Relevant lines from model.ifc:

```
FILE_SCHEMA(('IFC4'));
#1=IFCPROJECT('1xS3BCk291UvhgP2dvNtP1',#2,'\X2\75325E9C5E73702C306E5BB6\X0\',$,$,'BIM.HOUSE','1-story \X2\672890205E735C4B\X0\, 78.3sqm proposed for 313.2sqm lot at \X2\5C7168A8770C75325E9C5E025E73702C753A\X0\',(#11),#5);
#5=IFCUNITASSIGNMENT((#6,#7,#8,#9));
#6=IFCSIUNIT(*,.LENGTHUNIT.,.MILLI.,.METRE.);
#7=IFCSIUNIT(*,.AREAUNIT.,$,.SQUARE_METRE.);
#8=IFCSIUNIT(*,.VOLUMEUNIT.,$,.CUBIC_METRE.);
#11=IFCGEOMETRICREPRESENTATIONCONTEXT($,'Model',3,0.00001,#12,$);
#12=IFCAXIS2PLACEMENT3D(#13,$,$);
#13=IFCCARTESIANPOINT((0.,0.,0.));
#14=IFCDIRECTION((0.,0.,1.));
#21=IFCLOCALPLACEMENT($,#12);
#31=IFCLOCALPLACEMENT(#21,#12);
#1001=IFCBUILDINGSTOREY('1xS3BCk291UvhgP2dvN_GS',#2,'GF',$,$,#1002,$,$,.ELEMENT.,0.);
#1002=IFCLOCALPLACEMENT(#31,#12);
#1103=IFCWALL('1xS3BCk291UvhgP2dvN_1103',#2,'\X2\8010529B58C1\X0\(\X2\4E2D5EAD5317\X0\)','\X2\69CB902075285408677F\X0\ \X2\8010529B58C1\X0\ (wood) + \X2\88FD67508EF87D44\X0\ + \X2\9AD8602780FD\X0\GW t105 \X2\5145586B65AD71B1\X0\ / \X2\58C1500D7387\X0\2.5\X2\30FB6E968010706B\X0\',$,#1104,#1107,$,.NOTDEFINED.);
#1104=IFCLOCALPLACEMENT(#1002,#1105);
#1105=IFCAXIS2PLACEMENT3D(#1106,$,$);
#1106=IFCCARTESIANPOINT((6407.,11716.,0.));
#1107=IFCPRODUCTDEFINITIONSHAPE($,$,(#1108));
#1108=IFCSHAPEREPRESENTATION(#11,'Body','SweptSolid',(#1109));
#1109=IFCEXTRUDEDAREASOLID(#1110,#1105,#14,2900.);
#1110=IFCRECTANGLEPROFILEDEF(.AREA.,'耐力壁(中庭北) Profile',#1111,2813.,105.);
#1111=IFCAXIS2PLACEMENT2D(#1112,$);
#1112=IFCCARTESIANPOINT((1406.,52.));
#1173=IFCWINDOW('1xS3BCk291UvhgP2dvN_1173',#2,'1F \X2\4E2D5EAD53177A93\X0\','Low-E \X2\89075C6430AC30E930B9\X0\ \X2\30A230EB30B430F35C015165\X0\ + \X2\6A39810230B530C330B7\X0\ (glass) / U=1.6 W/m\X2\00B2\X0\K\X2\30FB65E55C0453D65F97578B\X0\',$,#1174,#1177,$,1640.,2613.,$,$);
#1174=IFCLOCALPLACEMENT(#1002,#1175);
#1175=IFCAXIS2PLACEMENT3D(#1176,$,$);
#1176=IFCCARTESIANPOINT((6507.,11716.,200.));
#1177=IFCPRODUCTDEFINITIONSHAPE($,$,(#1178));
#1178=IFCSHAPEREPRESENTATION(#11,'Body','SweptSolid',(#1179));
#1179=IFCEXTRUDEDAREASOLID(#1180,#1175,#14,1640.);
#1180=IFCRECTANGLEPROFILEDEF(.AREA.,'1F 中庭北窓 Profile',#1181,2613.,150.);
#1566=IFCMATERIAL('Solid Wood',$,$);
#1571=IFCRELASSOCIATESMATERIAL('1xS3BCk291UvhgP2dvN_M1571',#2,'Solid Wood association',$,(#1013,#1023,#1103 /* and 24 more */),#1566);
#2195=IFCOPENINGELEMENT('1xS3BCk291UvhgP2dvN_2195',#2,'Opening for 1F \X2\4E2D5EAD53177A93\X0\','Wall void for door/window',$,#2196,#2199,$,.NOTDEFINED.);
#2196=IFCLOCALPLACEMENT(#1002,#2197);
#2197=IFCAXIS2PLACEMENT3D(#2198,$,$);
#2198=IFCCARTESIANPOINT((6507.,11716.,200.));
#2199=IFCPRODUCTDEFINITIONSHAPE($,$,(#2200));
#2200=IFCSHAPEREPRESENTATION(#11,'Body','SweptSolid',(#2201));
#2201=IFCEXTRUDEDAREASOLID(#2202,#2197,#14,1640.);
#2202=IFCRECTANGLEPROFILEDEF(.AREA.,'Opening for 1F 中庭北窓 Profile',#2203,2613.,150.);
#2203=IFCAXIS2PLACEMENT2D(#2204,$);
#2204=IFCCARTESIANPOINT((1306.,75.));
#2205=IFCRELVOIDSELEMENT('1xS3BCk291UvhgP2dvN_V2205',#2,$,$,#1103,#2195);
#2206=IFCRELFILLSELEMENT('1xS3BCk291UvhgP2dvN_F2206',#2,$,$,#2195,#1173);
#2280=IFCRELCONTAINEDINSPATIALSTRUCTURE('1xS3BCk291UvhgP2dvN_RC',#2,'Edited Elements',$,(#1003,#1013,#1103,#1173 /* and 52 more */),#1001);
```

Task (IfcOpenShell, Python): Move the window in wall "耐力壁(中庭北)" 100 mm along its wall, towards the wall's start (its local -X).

```python
import ifcopenshell
import ifcopenshell.api.geometry
import ifcopenshell.util.placement
import ifcopenshell.util.unit

model = ifcopenshell.open("model.ifc")
unit_scale = ifcopenshell.util.unit.calculate_unit_scale(model)

window = model.by_guid("1xS3BCk291UvhgP2dvN_1173")
opening = window.FillsVoids[0].RelatingOpeningElement
wall = opening.VoidsElements[0].RelatingBuildingElement

wall_matrix = ifcopenshell.util.placement.get_local_placement(wall.ObjectPlacement)
shift = wall_matrix[:3, 0] * -0.1 / unit_scale
before = ifcopenshell.util.placement.get_local_placement(window.ObjectPlacement)[:3, 3].copy()

# The window is not placed relative to its opening, so move both.
for product in (opening, window):
    matrix = ifcopenshell.util.placement.get_local_placement(product.ObjectPlacement)
    matrix[:3, 3] += shift
    ifcopenshell.api.geometry.edit_object_placement(model, product=product, matrix=matrix, is_si=False)

after = ifcopenshell.util.placement.get_local_placement(window.ObjectPlacement)[:3, 3]
print("window moved by", (after - before).round(3) + 0.0)

model.write("model-out.ifc")
```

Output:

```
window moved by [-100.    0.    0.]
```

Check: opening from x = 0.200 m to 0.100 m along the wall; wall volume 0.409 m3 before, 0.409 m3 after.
